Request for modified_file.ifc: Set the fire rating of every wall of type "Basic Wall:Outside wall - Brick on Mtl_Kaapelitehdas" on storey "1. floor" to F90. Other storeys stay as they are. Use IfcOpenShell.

First a look at what the model holds.

```python
import ifcopenshell
import ifcopenshell.util.element

model = ifcopenshell.open("modified_file.ifc")
print(model.schema)
storey = next(s for s in model.by_type("IfcBuildingStorey") if s.Name == "1. floor")
walls = [e for e in ifcopenshell.util.element.get_decomposition(storey) if e.is_a("IfcWall")]
seen = {}
for e in walls:
    element_type = ifcopenshell.util.element.get_type(e)
    key = (element_type.Name if element_type != e and element_type else None, ifcopenshell.util.element.get_pset(e, "Pset_WallCommon", "FireRating"))
    seen[key] = seen.get(key, 0) + 1
for (name, value), count in sorted(seen.items(), key=str):
    print(count, "x", name, "|", value)
```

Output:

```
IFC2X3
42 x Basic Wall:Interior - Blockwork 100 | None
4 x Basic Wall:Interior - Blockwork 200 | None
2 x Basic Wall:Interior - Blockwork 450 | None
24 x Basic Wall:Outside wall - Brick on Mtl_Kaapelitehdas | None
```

```python
import ifcopenshell
import ifcopenshell.api.pset
import ifcopenshell.util.element

model = ifcopenshell.open("modified_file.ifc")

storey = next(s for s in model.by_type("IfcBuildingStorey") if s.Name == "1. floor")
walls = [e for e in ifcopenshell.util.element.get_decomposition(storey) if e.is_a("IfcWall")]

count = 0
for e in walls:
    element_type = ifcopenshell.util.element.get_type(e)
    if element_type in (None, e) or element_type.Name != "Basic Wall:Outside wall - Brick on Mtl_Kaapelitehdas":
        continue
    # add_pset returns the element's existing set when there is one.
    pset = ifcopenshell.api.pset.add_pset(model, product=e, name="Pset_WallCommon")
    ifcopenshell.api.pset.edit_pset(model, pset=pset, properties={"FireRating": "F90"})
    count += 1

print(count, "walls updated")

model.write("modified_file-out.ifc")
```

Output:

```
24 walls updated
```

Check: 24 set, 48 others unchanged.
